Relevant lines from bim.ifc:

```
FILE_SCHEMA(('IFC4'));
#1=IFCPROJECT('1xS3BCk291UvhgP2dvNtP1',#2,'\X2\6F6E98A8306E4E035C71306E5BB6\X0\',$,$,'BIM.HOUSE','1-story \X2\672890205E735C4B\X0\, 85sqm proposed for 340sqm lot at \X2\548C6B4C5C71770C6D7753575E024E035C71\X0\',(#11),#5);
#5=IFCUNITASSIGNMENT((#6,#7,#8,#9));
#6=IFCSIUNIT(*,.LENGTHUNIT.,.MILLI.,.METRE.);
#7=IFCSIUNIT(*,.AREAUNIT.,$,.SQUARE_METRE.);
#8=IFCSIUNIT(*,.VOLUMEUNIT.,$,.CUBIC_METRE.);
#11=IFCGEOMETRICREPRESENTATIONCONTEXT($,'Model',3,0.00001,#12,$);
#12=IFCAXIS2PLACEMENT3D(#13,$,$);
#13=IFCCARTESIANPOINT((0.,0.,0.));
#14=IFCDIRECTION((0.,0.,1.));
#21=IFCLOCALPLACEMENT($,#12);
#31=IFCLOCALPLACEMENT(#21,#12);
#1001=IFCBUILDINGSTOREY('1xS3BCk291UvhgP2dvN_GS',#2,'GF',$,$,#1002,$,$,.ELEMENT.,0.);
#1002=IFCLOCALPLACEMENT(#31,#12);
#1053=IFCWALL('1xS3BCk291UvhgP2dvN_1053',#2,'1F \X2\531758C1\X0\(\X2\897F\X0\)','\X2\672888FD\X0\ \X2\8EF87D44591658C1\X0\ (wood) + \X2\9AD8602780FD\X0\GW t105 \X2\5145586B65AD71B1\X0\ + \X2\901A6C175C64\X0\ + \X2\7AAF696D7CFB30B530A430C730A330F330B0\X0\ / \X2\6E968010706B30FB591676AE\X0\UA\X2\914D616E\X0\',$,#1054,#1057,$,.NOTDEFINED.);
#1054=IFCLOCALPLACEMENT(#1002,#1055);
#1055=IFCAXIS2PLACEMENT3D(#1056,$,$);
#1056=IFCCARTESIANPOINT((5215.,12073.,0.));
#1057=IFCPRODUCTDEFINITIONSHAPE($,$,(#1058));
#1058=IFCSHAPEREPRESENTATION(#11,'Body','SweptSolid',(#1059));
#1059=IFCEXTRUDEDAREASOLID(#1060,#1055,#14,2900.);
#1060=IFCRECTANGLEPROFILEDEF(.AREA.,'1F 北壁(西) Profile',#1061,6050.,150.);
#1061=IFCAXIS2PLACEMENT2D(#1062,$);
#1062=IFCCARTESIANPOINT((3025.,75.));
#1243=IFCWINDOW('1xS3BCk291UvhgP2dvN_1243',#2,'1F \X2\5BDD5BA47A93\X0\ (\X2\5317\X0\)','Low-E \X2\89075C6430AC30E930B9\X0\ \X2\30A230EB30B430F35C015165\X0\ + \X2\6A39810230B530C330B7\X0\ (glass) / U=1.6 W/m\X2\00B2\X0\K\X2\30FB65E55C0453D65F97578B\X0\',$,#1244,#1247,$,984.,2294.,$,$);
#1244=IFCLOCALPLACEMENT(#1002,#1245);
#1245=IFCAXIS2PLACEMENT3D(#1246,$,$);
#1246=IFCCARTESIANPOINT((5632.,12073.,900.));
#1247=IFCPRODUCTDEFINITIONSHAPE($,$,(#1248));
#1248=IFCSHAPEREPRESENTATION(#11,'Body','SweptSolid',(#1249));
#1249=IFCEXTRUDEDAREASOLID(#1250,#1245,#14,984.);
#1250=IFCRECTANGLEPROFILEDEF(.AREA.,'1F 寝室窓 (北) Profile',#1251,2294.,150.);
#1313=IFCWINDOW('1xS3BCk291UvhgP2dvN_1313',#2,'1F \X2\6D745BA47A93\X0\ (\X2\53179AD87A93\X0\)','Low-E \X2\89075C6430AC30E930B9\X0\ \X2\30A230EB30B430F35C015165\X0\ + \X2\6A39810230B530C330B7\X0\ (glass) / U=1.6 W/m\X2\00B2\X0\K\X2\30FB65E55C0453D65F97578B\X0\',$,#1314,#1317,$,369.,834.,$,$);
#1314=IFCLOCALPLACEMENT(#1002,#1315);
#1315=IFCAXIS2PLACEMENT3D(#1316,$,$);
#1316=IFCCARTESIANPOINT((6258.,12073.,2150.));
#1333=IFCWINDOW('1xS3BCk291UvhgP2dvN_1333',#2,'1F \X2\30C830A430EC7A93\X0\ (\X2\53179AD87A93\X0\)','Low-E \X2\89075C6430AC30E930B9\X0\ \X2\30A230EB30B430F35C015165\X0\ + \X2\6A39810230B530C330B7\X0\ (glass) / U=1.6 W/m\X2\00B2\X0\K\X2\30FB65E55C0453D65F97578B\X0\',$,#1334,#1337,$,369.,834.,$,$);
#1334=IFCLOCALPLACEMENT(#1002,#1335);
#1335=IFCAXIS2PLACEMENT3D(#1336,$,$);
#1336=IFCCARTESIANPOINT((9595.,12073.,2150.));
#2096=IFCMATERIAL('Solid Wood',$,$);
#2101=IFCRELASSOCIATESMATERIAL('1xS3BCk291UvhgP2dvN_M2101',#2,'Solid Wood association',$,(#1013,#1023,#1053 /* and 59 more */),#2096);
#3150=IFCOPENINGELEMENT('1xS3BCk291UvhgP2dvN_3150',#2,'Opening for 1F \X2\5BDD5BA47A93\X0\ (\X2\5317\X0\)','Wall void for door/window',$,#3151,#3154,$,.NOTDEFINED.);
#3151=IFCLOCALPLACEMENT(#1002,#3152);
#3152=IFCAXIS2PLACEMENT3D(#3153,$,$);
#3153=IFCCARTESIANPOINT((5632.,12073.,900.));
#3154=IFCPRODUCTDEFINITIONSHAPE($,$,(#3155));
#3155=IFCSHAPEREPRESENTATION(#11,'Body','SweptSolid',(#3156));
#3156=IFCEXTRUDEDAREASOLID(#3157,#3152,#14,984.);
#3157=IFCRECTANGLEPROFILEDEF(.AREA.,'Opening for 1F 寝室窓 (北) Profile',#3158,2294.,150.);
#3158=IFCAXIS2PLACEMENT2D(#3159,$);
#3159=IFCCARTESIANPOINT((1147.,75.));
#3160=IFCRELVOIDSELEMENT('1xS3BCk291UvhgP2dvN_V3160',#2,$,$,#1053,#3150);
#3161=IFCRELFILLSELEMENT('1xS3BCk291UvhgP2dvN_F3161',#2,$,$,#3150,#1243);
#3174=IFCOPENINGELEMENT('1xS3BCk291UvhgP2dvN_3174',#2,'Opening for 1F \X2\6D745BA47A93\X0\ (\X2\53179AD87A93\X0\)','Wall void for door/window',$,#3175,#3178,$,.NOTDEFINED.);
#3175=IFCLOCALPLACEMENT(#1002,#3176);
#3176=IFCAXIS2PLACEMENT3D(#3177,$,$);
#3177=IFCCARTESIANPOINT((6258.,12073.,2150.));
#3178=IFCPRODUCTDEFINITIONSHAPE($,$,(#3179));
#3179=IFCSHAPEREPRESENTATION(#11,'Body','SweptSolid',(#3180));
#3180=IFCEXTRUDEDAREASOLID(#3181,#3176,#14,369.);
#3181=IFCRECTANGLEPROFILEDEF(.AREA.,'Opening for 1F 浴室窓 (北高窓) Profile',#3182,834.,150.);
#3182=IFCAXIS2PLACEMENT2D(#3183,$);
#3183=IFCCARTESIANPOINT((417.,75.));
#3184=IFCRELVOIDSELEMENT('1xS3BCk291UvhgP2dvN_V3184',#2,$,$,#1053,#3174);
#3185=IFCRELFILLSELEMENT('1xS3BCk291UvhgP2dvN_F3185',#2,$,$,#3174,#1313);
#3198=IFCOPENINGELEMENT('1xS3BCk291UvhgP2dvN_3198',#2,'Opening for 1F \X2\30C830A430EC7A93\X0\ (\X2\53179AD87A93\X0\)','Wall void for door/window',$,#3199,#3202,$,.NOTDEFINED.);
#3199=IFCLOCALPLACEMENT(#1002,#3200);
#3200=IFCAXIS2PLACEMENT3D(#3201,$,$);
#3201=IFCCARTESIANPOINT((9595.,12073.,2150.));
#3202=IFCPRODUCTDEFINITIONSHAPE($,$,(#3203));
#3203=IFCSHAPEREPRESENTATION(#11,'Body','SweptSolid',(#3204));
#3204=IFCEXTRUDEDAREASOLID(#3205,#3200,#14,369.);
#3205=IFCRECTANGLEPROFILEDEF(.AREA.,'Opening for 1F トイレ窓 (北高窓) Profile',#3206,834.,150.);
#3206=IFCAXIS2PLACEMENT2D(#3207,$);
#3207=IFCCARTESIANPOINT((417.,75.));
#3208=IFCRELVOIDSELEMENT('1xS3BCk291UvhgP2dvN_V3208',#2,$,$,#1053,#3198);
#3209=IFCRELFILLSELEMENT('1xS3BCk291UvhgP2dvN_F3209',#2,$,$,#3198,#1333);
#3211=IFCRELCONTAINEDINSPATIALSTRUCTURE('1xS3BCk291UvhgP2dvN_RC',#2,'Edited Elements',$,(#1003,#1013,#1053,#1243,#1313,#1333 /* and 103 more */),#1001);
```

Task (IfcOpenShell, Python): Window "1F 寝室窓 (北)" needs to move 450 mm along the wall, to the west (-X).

```python
import ifcopenshell
import ifcopenshell.api.geometry
import ifcopenshell.util.placement

model = ifcopenshell.open("bim.ifc")

window = model.by_id(1243)
opening = window.FillsVoids[0].RelatingOpeningElement
wall = opening.VoidsElements[0].RelatingBuildingElement

wall_matrix = ifcopenshell.util.placement.get_local_placement(wall.ObjectPlacement)
shift = wall_matrix[:3, 0] * -450.0
before = ifcopenshell.util.placement.get_local_placement(window.ObjectPlacement)[:3, 3].copy()

# The window is not placed relative to its opening, so move both.
for product in (opening, window):
    matrix = ifcopenshell.util.placement.get_local_placement(product.ObjectPlacement)
    matrix[:3, 3] += shift
    ifcopenshell.api.geometry.edit_object_placement(model, product=product, matrix=matrix, is_si=False)

after = ifcopenshell.util.placement.get_local_placement(window.ObjectPlacement)[:3, 3]
print("window moved by", (after - before).round(3) + 0.0)

model.write("bim_rev.ifc")
```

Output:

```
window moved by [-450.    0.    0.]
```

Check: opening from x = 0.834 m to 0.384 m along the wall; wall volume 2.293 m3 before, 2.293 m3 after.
